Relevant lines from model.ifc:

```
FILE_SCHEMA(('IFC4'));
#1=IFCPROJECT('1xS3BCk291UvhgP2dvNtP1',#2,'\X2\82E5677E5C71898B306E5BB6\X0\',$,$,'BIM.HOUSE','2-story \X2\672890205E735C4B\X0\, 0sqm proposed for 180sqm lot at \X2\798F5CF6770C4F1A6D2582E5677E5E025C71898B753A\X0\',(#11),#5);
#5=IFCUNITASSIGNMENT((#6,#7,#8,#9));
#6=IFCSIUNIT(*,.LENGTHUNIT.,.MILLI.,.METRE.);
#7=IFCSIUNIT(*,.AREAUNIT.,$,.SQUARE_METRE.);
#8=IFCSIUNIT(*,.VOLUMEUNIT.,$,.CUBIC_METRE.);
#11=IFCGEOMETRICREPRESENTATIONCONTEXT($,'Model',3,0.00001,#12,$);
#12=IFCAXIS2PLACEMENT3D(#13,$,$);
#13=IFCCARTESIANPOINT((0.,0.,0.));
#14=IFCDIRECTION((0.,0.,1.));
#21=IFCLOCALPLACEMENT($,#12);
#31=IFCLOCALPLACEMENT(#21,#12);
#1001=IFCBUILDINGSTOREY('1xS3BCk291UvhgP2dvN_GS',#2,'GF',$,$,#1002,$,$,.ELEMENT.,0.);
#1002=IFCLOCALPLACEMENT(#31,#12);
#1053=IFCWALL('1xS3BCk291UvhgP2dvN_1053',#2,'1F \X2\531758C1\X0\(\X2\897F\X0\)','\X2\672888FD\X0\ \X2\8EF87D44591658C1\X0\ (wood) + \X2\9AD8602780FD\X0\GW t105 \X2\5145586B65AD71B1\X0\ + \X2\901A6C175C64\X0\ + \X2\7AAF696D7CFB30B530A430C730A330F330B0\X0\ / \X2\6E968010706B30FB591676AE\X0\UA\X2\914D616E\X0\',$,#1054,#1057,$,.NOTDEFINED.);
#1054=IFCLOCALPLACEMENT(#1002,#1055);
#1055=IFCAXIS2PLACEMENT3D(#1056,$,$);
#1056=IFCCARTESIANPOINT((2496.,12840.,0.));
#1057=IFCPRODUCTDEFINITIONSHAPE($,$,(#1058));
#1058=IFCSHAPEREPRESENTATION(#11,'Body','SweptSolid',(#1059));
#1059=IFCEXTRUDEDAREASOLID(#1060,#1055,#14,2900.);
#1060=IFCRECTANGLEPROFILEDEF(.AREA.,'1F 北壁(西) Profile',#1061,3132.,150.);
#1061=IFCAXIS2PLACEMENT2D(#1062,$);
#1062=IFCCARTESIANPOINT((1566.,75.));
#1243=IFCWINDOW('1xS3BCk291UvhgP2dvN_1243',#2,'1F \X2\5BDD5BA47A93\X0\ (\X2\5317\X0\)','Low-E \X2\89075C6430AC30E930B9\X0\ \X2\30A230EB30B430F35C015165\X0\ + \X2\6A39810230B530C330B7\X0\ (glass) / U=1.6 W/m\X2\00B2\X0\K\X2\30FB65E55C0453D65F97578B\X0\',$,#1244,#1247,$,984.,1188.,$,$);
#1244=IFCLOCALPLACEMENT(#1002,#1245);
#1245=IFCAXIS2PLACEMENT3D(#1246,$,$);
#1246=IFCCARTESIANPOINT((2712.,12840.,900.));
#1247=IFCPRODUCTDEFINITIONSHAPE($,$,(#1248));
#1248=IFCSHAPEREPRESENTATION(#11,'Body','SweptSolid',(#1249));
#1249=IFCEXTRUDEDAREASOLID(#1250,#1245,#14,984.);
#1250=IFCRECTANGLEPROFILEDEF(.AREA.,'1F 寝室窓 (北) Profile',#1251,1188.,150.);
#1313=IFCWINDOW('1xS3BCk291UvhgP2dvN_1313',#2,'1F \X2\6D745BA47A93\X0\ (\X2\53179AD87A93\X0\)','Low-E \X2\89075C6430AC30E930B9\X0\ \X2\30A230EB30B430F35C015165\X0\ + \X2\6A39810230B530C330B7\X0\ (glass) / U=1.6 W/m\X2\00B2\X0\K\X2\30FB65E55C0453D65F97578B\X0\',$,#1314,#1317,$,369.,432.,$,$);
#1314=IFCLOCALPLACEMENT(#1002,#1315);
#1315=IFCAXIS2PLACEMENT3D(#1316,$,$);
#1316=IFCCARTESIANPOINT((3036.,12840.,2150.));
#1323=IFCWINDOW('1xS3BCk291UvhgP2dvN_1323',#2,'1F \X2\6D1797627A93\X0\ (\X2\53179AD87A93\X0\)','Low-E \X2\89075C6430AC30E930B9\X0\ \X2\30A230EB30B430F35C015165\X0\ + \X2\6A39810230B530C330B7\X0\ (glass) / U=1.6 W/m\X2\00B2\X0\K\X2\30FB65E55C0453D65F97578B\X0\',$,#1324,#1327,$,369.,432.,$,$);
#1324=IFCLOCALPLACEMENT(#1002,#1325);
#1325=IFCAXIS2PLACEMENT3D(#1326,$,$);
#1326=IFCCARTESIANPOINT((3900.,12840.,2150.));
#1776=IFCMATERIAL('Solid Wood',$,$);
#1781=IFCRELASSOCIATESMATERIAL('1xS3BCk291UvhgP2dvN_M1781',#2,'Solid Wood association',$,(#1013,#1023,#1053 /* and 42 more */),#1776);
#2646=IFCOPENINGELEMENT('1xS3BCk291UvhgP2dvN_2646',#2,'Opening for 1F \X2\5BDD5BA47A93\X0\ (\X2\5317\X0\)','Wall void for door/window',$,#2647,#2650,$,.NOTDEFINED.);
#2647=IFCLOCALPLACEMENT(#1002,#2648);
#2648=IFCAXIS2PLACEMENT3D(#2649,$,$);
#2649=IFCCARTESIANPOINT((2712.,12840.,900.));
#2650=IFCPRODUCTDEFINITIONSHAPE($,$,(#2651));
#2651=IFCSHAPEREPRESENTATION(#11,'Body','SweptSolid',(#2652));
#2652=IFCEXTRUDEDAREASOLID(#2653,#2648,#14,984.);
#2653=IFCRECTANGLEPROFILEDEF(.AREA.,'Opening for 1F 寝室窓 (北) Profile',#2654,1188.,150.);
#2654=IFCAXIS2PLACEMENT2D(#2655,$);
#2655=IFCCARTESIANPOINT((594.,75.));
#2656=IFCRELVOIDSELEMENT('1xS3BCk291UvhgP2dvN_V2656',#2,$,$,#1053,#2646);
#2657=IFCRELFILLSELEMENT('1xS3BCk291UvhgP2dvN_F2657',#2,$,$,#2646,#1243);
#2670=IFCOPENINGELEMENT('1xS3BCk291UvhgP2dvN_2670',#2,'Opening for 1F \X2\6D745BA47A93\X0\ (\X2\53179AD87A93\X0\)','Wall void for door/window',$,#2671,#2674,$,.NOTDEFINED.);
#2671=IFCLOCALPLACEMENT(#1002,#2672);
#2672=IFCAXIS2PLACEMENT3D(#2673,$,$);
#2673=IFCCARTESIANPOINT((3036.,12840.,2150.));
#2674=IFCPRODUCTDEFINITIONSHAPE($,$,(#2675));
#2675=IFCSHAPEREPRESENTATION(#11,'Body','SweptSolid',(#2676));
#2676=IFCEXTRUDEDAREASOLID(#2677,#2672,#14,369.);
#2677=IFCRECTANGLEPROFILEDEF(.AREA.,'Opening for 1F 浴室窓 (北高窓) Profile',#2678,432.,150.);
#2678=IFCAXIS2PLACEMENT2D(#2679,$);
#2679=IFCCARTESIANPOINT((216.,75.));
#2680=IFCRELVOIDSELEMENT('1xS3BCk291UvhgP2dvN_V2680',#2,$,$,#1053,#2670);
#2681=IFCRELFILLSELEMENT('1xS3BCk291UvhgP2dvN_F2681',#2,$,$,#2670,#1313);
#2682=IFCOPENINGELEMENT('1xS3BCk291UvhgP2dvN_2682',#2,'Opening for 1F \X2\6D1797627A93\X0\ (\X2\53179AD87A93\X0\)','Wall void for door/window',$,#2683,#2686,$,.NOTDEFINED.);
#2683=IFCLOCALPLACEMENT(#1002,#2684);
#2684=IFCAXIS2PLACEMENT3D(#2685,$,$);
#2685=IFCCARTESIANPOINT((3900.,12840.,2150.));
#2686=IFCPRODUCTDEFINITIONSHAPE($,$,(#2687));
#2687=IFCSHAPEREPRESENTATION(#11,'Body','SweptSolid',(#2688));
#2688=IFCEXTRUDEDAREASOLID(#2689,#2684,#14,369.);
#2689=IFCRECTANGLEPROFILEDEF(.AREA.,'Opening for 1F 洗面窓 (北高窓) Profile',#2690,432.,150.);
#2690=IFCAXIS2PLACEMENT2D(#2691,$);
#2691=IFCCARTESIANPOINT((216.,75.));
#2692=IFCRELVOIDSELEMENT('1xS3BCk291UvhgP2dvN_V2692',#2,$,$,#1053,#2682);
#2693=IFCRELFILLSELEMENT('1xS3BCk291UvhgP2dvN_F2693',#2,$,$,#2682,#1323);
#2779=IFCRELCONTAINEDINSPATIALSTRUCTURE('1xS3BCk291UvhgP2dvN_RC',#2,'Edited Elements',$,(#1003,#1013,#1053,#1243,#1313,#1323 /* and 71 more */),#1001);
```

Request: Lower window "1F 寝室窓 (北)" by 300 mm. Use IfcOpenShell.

```python
import numpy as np
import ifcopenshell
import ifcopenshell.api.geometry
import ifcopenshell.util.placement
import ifcopenshell.util.unit

model = ifcopenshell.open("model.ifc")
unit_scale = ifcopenshell.util.unit.calculate_unit_scale(model)

window = model.by_guid("1xS3BCk291UvhgP2dvN_1243")
opening = window.FillsVoids[0].RelatingOpeningElement
dz = -300.0

shift = np.array([0.0, 0.0, dz])
# The window is not placed relative to its opening, so move both.
for product in (opening, window):
    matrix = ifcopenshell.util.placement.get_local_placement(product.ObjectPlacement)
    matrix[:3, 3] += shift
    ifcopenshell.api.geometry.edit_object_placement(model, product=product, matrix=matrix, is_si=False)

print(f"moved by {dz * unit_scale:+.3f} m")

model.write("model_edited.ifc")
```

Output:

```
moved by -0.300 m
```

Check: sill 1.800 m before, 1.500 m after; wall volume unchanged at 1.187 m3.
